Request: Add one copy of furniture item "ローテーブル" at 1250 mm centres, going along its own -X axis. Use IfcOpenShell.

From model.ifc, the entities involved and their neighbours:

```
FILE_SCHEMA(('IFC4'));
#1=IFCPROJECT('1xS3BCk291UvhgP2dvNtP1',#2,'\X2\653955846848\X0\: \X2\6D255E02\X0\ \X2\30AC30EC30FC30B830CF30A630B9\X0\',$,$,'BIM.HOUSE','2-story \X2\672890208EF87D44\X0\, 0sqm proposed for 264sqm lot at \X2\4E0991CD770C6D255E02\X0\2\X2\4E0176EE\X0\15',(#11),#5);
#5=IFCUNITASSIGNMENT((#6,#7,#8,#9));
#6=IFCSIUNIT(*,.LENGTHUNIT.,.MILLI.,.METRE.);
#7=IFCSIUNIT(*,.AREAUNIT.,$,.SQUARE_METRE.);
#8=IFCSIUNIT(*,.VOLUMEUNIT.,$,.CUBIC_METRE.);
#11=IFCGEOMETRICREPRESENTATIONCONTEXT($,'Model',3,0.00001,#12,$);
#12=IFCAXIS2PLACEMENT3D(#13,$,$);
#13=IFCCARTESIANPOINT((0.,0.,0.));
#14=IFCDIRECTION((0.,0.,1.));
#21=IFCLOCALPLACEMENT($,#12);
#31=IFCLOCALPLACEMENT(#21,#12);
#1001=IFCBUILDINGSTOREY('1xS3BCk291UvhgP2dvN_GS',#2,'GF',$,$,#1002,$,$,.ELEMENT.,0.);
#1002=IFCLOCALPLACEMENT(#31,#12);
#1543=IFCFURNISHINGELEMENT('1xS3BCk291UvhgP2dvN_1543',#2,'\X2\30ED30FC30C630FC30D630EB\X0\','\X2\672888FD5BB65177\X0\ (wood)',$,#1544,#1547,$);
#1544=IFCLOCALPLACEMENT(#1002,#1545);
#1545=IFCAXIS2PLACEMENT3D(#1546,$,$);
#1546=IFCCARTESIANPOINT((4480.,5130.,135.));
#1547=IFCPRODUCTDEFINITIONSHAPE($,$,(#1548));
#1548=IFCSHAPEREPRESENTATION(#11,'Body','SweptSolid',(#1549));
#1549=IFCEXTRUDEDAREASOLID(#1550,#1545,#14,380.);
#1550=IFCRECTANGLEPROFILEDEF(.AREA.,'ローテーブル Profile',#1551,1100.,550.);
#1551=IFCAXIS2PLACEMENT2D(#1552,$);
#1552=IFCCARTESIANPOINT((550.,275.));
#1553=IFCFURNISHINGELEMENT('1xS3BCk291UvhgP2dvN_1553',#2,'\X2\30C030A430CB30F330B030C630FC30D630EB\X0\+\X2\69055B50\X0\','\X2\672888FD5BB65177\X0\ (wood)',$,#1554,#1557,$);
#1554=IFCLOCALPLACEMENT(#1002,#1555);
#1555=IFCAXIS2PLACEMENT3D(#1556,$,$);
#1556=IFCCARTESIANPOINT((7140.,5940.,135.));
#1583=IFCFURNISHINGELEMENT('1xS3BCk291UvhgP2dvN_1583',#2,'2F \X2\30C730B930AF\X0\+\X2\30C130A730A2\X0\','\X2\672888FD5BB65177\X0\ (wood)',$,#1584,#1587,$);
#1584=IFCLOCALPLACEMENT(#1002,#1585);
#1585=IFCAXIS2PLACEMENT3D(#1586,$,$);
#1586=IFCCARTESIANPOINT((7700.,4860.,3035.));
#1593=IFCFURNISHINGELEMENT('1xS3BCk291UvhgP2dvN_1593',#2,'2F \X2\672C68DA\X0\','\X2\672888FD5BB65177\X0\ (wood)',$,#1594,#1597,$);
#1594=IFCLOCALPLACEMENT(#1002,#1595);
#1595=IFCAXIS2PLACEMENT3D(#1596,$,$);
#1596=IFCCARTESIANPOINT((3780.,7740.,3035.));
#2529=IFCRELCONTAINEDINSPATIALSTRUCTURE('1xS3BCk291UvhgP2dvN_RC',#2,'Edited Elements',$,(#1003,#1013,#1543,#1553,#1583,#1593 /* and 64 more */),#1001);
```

```python
import ifcopenshell
import ifcopenshell.api.geometry
import ifcopenshell.api.root
import ifcopenshell.util.element
import ifcopenshell.util.placement
import ifcopenshell.util.unit

model = ifcopenshell.open("model.ifc")
unit_scale = ifcopenshell.util.unit.calculate_unit_scale(model)


def reuse_history(source, copy):
    """copy_class also copies each property set's owner history, people and application; keep the originals."""
    for rel in copy.IsDefinedBy:
        if rel.is_a("IfcRelDefinesByProperties") and (history := rel.RelatingPropertyDefinition.OwnerHistory):
            rel.RelatingPropertyDefinition.OwnerHistory = source.OwnerHistory
            ifcopenshell.util.element.remove_deep2(model, history)


source = model.by_id(1543)
base = ifcopenshell.util.placement.get_local_placement(source.ObjectPlacement)
step = -base[:3, 0] * 1.25 / unit_scale

for i in range(1, 2):
    copy = ifcopenshell.api.root.copy_class(model, product=source)
    copy.Representation = ifcopenshell.util.element.copy_deep(
        model, source.Representation, exclude=["IfcGeometricRepresentationContext", "IfcRepresentationMap"]
    )
    reuse_history(source, copy)
    matrix = base.copy()
    matrix[:3, 3] += i * step
    print("added at", matrix[:3, 3].round(3) + 0.0)
    ifcopenshell.api.geometry.edit_object_placement(model, product=copy, matrix=matrix, is_si=False)

model.write("model-out.ifc")
```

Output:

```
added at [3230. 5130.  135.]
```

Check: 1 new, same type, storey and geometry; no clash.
